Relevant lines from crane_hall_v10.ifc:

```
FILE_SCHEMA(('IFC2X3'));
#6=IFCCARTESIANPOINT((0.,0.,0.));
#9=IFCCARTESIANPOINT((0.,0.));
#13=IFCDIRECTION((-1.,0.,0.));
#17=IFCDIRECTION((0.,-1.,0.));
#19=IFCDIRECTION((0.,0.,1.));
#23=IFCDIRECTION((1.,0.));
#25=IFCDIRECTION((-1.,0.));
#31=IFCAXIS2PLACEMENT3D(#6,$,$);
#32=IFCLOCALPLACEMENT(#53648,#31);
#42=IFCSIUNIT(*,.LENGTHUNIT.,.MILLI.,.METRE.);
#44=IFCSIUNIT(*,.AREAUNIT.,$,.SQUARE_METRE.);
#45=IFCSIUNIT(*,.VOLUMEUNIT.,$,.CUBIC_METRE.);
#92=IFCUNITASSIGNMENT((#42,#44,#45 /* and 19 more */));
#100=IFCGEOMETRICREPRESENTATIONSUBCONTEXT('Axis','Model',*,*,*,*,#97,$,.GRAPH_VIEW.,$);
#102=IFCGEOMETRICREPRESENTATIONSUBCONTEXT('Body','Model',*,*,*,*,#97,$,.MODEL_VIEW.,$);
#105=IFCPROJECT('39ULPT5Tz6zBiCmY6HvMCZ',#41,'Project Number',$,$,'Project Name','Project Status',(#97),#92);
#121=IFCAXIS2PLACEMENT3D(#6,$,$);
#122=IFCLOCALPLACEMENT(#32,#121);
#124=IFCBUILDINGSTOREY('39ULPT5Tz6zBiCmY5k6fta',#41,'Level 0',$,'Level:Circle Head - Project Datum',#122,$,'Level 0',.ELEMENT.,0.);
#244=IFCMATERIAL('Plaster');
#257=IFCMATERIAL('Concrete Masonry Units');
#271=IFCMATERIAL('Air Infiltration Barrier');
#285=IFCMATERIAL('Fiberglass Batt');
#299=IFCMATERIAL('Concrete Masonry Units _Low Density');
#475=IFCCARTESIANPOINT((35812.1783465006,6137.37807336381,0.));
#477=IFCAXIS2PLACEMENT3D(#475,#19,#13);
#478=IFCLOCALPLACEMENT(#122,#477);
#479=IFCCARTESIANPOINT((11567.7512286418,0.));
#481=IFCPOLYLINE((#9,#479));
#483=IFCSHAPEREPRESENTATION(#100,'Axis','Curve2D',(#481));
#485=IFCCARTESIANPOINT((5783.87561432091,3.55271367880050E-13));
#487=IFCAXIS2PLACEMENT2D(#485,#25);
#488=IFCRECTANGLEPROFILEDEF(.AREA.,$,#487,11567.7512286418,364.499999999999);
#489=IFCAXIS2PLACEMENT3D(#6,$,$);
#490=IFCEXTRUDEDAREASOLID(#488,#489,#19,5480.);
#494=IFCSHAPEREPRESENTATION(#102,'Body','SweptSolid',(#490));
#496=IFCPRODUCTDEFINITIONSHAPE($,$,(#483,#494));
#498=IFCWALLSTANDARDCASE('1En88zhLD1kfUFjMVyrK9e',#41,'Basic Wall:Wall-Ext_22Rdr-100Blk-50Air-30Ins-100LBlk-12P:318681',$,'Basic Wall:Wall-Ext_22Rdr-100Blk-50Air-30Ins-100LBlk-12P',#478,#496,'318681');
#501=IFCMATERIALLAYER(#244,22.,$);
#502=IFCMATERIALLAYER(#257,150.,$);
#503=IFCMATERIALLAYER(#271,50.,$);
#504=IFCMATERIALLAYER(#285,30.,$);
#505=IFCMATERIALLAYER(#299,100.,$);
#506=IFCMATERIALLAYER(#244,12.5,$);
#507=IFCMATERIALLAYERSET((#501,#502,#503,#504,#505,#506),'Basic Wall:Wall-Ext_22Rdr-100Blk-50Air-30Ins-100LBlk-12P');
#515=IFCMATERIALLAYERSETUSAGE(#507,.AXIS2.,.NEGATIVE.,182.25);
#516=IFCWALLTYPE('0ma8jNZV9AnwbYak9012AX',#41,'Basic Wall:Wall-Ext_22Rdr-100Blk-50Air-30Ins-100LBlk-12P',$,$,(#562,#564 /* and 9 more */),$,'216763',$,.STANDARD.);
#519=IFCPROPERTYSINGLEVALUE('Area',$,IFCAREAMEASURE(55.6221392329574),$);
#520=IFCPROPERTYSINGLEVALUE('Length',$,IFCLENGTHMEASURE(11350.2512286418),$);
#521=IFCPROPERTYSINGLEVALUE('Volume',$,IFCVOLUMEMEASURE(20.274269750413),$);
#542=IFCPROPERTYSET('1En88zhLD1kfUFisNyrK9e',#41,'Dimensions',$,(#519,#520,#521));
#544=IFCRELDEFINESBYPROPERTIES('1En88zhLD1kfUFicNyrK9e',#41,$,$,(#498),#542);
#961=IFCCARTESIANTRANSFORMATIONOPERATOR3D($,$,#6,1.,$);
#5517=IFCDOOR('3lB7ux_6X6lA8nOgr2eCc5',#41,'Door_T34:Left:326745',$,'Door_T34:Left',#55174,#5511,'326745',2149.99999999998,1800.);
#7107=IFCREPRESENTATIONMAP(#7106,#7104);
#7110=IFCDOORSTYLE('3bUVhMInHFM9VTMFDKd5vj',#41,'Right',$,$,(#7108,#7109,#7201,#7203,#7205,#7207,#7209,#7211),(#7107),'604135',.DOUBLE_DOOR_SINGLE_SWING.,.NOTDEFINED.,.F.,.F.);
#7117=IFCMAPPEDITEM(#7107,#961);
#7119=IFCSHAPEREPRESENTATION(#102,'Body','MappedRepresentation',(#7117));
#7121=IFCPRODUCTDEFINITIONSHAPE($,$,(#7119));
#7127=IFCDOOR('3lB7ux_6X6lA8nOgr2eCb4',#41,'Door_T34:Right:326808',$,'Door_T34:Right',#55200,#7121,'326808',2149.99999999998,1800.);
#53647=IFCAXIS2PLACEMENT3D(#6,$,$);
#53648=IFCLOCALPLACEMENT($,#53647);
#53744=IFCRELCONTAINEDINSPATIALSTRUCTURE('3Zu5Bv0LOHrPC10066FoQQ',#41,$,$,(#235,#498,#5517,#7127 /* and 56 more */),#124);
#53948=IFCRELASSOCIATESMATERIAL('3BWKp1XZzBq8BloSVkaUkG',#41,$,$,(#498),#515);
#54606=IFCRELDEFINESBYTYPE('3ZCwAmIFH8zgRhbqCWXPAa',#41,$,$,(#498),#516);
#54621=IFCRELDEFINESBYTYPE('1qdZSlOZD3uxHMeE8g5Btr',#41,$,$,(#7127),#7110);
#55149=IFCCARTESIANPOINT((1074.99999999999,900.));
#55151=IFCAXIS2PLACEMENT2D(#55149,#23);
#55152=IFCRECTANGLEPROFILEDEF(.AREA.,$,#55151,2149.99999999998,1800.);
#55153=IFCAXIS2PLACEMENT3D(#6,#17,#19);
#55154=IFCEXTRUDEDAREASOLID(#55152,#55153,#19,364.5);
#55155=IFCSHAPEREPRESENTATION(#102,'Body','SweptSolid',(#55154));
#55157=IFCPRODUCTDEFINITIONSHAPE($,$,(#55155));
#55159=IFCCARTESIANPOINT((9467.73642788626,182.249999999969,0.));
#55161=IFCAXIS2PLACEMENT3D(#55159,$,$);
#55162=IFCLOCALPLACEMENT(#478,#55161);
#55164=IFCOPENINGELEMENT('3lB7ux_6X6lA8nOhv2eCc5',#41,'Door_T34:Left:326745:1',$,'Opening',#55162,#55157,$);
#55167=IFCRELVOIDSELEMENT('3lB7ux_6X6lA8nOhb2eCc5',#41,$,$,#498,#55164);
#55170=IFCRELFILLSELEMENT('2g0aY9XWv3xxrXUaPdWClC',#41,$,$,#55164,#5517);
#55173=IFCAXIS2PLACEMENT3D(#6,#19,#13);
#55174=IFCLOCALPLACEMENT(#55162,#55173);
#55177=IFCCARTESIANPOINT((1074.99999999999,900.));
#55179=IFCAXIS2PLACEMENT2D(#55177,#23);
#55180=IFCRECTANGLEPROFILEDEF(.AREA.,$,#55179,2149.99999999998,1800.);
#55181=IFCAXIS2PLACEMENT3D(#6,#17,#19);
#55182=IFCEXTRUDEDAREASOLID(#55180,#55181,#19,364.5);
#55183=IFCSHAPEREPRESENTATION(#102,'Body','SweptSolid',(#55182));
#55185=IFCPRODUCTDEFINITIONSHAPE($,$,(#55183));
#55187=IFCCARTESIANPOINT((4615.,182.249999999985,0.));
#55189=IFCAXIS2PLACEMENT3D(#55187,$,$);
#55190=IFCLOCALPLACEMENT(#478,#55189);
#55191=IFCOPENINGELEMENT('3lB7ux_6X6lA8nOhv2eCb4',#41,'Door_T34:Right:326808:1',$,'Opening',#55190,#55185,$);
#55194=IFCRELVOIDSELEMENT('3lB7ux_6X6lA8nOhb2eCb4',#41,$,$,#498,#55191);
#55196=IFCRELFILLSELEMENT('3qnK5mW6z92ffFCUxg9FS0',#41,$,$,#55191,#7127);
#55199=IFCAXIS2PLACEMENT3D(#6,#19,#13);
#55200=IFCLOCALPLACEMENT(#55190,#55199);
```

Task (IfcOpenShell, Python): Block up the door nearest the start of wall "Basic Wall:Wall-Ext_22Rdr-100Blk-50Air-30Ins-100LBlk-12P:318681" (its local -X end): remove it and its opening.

```python
import ifcopenshell
import ifcopenshell.api.feature
import ifcopenshell.api.pset
import ifcopenshell.api.root
import ifcopenshell.geom
import ifcopenshell.util.element
import ifcopenshell.util.shape
import ifcopenshell.util.unit

model = ifcopenshell.open("crane_hall_v10.ifc")
area_scale = ifcopenshell.util.unit.calculate_unit_scale(model, "AREAUNIT")
volume_scale = ifcopenshell.util.unit.calculate_unit_scale(model, "VOLUMEUNIT")
settings = ifcopenshell.geom.settings()


def volume(element):
    """Net volume in cubic metres, openings subtracted."""
    shape = ifcopenshell.geom.create_shape(settings, element)
    return ifcopenshell.util.shape.get_volume(shape.geometry)


door = model.by_guid("3lB7ux_6X6lA8nOgr2eCb4")
opening = door.FillsVoids[0].RelatingOpeningElement
wall = opening.VoidsElements[0].RelatingBuildingElement
before = volume(wall)

ifcopenshell.api.root.remove_product(model, product=door)
ifcopenshell.api.feature.remove_feature(model, feature=opening)

after = volume(wall)
thickness = 0.3645  # wall thickness in metres

# Update the wall's stored quantities.
pset = model.by_id(ifcopenshell.util.element.get_pset(wall, "Dimensions", should_inherit=False)["id"])
ifcopenshell.api.pset.edit_pset(model, pset=pset, properties={
    "Area": model.create_entity("IfcAreaMeasure", after / thickness / area_scale),
    "Volume": model.create_entity("IfcVolumeMeasure", after / volume_scale),
})

print(f"wall volume {before:.3f} -> {after:.3f} m3")

model.write("crane_hall_v10_v2.ifc")
```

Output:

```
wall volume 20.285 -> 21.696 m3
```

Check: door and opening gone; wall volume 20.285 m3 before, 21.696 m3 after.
